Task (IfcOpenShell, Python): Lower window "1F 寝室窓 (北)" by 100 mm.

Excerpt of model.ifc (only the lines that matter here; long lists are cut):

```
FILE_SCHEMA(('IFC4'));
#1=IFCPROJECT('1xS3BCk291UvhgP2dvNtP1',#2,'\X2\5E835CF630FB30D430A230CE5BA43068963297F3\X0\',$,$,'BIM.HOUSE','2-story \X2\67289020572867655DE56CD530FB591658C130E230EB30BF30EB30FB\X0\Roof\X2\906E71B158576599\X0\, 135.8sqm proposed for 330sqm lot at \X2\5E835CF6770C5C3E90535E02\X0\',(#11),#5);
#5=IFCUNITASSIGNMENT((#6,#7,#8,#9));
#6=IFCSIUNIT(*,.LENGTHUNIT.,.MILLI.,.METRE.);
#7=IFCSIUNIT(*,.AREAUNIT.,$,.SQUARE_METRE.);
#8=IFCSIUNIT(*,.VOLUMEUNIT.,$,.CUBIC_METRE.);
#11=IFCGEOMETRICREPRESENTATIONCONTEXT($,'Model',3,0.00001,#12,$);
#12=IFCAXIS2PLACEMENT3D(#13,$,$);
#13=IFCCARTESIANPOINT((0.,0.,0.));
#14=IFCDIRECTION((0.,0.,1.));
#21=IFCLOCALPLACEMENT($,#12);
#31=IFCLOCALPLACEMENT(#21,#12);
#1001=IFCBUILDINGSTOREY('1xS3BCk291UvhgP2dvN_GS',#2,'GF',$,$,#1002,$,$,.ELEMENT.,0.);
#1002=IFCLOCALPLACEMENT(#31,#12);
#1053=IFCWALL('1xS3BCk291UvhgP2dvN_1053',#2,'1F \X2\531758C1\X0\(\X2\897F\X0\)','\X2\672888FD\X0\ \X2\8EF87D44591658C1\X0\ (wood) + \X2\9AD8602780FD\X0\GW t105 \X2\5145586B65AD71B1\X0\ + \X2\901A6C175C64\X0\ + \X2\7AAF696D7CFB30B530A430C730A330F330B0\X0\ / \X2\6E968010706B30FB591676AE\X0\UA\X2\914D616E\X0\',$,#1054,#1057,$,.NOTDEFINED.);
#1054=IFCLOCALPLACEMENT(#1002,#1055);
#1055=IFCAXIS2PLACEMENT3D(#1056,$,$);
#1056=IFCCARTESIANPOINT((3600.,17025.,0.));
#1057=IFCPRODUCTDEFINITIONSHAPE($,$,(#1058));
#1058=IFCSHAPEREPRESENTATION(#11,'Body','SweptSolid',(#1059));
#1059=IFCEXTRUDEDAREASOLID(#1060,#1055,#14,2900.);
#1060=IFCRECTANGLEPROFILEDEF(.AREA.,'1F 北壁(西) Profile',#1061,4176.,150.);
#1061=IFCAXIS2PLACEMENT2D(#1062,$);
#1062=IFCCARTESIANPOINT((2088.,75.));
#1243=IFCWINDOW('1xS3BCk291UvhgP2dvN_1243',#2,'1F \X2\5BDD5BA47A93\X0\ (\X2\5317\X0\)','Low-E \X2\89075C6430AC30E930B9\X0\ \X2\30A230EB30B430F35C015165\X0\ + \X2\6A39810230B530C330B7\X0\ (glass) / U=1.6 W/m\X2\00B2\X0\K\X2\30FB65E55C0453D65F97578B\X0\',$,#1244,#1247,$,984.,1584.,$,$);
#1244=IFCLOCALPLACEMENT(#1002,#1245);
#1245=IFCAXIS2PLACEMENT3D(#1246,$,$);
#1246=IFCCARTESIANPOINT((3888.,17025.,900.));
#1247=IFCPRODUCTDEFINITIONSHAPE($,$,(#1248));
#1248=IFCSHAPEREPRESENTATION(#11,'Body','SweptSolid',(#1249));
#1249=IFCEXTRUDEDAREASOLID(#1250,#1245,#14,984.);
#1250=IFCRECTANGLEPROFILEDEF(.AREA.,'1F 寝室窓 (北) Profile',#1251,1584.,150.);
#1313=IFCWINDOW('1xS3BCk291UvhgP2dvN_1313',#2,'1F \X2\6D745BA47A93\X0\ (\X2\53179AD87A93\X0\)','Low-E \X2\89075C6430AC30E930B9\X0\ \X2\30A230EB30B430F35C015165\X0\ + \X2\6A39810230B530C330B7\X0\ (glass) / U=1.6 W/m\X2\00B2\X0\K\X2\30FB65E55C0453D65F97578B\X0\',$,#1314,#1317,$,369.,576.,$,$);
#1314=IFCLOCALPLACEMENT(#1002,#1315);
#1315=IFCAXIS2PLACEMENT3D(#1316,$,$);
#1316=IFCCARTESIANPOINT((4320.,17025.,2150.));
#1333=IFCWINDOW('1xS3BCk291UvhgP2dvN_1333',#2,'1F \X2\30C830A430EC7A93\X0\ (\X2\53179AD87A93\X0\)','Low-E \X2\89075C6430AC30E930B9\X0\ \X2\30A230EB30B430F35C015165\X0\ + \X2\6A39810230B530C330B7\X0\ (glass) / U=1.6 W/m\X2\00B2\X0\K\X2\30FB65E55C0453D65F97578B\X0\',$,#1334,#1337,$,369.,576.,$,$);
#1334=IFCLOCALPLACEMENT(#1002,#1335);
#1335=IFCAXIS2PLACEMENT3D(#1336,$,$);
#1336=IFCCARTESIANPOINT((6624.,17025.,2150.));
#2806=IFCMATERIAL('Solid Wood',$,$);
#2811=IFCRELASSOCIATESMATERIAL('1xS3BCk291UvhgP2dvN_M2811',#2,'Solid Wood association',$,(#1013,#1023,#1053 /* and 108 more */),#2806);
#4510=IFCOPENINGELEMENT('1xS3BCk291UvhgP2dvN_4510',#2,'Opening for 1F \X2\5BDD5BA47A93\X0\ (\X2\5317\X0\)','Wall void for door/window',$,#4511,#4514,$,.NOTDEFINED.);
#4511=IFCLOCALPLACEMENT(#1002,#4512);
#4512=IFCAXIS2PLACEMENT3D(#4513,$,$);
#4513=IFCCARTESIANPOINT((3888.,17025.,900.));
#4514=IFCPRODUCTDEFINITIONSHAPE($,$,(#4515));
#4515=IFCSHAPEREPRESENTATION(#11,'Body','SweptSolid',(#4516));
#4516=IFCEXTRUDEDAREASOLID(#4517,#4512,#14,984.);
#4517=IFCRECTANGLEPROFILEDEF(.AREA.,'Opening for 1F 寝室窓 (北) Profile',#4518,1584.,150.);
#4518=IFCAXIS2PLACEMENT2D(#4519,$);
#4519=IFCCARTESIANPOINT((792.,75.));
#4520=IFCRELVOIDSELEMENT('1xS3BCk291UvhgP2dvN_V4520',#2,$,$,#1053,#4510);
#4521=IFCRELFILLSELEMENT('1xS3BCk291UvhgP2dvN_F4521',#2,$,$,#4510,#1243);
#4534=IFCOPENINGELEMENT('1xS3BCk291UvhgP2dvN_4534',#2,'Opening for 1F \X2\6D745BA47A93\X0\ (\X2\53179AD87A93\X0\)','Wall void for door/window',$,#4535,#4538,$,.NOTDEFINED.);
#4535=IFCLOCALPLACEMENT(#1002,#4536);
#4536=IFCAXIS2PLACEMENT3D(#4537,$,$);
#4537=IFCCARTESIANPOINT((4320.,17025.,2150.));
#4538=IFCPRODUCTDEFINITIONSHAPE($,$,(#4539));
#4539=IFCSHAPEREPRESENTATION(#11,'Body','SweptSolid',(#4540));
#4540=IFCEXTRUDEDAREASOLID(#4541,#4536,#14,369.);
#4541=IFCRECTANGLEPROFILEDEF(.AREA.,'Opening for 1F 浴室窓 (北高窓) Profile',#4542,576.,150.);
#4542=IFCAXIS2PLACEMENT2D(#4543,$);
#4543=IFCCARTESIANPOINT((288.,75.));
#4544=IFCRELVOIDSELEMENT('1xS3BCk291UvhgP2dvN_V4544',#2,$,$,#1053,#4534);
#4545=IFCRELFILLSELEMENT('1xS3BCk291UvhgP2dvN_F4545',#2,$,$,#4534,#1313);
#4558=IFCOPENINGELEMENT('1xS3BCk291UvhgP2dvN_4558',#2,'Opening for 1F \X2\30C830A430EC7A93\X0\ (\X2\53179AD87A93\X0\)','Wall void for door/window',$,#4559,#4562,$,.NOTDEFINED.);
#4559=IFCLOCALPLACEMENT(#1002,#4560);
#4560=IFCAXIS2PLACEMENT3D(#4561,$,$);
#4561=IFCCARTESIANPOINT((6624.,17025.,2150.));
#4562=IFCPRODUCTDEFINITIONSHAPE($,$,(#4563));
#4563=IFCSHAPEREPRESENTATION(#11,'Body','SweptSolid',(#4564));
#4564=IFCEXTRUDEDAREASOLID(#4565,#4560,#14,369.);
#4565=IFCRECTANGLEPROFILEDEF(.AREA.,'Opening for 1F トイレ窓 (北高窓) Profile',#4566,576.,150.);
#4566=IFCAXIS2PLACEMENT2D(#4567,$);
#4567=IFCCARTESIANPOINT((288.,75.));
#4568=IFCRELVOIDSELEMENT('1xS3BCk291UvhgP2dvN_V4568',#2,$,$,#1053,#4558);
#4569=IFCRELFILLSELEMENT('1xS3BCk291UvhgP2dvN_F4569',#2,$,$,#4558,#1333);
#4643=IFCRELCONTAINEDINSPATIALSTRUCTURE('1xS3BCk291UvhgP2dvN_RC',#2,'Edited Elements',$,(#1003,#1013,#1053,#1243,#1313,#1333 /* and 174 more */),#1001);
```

```python
import numpy as np
import ifcopenshell
import ifcopenshell.api.geometry
import ifcopenshell.util.placement
import ifcopenshell.util.unit

model = ifcopenshell.open("model.ifc")
unit_scale = ifcopenshell.util.unit.calculate_unit_scale(model)

window = model.by_guid("1xS3BCk291UvhgP2dvN_1243")
opening = window.FillsVoids[0].RelatingOpeningElement
dz = -100.0

shift = np.array([0.0, 0.0, dz])
# The window is not placed relative to its opening, so move both.
for product in (opening, window):
    matrix = ifcopenshell.util.placement.get_local_placement(product.ObjectPlacement)
    matrix[:3, 3] += shift
    ifcopenshell.api.geometry.edit_object_placement(model, product=product, matrix=matrix, is_si=False)

print(f"moved by {dz * unit_scale:+.3f} m")

model.write("model_rev.ifc")
```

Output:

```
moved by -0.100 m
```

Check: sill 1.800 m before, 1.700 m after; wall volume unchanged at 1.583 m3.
